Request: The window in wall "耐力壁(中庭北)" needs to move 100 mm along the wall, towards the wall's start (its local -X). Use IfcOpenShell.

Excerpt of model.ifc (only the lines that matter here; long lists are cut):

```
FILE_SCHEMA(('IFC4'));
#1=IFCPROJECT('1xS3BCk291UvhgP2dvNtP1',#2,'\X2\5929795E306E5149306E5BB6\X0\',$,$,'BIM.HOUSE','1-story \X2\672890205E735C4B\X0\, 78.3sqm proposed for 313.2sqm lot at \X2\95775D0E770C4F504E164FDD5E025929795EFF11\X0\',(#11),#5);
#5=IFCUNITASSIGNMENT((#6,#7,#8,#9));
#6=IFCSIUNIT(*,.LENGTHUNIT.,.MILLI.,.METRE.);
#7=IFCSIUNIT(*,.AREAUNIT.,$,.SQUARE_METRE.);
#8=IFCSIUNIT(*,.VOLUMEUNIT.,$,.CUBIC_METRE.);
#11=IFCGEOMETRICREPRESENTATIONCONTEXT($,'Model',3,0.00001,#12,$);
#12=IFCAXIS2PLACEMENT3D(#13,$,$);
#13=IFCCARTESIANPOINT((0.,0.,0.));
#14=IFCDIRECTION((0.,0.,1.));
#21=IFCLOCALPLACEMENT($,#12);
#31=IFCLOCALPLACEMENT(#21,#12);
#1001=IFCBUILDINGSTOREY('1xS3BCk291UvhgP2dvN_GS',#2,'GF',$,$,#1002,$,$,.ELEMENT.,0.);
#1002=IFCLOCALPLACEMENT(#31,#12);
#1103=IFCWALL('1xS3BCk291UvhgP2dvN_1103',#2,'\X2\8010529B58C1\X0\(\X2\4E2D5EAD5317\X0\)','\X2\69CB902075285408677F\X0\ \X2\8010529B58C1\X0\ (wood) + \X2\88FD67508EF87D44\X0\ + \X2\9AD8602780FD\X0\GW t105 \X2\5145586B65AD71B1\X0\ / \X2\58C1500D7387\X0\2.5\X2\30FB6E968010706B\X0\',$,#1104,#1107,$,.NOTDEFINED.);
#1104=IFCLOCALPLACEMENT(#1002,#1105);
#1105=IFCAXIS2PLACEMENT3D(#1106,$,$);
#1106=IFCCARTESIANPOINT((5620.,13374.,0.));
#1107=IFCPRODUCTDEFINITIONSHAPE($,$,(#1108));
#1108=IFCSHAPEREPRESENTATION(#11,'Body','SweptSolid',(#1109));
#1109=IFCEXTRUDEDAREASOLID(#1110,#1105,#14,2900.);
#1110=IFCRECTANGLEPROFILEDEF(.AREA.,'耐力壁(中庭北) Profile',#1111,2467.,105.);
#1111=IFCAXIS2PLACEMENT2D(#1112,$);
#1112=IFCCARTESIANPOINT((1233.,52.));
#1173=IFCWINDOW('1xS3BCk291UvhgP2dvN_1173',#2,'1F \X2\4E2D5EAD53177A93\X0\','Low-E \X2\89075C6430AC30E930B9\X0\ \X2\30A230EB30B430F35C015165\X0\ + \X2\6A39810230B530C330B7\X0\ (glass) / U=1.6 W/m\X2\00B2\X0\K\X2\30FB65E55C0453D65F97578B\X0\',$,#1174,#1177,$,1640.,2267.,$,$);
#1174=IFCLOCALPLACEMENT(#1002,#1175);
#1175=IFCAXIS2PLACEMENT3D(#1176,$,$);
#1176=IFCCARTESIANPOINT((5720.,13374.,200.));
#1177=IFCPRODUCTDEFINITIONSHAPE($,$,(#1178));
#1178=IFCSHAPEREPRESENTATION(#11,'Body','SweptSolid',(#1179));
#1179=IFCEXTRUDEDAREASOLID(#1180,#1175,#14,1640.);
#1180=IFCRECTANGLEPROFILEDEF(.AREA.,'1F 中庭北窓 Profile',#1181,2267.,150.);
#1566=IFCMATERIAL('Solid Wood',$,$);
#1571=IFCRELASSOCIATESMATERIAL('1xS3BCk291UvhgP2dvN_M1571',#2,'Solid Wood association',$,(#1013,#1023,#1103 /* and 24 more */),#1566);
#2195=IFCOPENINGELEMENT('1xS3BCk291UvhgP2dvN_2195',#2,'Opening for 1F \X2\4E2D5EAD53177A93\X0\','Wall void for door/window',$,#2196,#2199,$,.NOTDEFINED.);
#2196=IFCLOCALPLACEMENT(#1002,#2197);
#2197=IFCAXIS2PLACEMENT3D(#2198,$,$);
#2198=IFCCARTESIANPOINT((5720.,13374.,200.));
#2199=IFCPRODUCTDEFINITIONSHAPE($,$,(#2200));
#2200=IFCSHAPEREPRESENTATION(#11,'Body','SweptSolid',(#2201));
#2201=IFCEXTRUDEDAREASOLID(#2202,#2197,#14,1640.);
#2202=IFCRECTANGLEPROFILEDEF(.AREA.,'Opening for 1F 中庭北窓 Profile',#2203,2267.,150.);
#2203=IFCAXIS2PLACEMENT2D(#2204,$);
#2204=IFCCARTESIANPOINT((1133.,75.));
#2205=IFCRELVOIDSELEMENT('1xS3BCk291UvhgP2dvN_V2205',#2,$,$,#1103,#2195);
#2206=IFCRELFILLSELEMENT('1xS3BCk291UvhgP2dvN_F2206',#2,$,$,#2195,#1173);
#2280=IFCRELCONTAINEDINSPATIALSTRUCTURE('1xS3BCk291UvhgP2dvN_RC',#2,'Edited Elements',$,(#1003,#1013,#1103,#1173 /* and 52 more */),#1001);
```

```python
import ifcopenshell
import ifcopenshell.api.geometry
import ifcopenshell.util.placement
import ifcopenshell.util.unit

model = ifcopenshell.open("model.ifc")
unit_scale = ifcopenshell.util.unit.calculate_unit_scale(model)

window = model.by_guid("1xS3BCk291UvhgP2dvN_1173")
opening = window.FillsVoids[0].RelatingOpeningElement
wall = opening.VoidsElements[0].RelatingBuildingElement

wall_matrix = ifcopenshell.util.placement.get_local_placement(wall.ObjectPlacement)
shift = wall_matrix[:3, 0] * -0.1 / unit_scale
before = ifcopenshell.util.placement.get_local_placement(window.ObjectPlacement)[:3, 3].copy()

# The window is not placed relative to its opening, so move both.
for product in (opening, window):
    matrix = ifcopenshell.util.placement.get_local_placement(product.ObjectPlacement)
    matrix[:3, 3] += shift
    ifcopenshell.api.geometry.edit_object_placement(model, product=product, matrix=matrix, is_si=False)

after = ifcopenshell.util.placement.get_local_placement(window.ObjectPlacement)[:3, 3]
print("window moved by", (after - before).round(3) + 0.0)

model.write("model_v2.ifc")
```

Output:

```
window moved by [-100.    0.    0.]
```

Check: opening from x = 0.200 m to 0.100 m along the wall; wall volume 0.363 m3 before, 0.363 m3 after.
